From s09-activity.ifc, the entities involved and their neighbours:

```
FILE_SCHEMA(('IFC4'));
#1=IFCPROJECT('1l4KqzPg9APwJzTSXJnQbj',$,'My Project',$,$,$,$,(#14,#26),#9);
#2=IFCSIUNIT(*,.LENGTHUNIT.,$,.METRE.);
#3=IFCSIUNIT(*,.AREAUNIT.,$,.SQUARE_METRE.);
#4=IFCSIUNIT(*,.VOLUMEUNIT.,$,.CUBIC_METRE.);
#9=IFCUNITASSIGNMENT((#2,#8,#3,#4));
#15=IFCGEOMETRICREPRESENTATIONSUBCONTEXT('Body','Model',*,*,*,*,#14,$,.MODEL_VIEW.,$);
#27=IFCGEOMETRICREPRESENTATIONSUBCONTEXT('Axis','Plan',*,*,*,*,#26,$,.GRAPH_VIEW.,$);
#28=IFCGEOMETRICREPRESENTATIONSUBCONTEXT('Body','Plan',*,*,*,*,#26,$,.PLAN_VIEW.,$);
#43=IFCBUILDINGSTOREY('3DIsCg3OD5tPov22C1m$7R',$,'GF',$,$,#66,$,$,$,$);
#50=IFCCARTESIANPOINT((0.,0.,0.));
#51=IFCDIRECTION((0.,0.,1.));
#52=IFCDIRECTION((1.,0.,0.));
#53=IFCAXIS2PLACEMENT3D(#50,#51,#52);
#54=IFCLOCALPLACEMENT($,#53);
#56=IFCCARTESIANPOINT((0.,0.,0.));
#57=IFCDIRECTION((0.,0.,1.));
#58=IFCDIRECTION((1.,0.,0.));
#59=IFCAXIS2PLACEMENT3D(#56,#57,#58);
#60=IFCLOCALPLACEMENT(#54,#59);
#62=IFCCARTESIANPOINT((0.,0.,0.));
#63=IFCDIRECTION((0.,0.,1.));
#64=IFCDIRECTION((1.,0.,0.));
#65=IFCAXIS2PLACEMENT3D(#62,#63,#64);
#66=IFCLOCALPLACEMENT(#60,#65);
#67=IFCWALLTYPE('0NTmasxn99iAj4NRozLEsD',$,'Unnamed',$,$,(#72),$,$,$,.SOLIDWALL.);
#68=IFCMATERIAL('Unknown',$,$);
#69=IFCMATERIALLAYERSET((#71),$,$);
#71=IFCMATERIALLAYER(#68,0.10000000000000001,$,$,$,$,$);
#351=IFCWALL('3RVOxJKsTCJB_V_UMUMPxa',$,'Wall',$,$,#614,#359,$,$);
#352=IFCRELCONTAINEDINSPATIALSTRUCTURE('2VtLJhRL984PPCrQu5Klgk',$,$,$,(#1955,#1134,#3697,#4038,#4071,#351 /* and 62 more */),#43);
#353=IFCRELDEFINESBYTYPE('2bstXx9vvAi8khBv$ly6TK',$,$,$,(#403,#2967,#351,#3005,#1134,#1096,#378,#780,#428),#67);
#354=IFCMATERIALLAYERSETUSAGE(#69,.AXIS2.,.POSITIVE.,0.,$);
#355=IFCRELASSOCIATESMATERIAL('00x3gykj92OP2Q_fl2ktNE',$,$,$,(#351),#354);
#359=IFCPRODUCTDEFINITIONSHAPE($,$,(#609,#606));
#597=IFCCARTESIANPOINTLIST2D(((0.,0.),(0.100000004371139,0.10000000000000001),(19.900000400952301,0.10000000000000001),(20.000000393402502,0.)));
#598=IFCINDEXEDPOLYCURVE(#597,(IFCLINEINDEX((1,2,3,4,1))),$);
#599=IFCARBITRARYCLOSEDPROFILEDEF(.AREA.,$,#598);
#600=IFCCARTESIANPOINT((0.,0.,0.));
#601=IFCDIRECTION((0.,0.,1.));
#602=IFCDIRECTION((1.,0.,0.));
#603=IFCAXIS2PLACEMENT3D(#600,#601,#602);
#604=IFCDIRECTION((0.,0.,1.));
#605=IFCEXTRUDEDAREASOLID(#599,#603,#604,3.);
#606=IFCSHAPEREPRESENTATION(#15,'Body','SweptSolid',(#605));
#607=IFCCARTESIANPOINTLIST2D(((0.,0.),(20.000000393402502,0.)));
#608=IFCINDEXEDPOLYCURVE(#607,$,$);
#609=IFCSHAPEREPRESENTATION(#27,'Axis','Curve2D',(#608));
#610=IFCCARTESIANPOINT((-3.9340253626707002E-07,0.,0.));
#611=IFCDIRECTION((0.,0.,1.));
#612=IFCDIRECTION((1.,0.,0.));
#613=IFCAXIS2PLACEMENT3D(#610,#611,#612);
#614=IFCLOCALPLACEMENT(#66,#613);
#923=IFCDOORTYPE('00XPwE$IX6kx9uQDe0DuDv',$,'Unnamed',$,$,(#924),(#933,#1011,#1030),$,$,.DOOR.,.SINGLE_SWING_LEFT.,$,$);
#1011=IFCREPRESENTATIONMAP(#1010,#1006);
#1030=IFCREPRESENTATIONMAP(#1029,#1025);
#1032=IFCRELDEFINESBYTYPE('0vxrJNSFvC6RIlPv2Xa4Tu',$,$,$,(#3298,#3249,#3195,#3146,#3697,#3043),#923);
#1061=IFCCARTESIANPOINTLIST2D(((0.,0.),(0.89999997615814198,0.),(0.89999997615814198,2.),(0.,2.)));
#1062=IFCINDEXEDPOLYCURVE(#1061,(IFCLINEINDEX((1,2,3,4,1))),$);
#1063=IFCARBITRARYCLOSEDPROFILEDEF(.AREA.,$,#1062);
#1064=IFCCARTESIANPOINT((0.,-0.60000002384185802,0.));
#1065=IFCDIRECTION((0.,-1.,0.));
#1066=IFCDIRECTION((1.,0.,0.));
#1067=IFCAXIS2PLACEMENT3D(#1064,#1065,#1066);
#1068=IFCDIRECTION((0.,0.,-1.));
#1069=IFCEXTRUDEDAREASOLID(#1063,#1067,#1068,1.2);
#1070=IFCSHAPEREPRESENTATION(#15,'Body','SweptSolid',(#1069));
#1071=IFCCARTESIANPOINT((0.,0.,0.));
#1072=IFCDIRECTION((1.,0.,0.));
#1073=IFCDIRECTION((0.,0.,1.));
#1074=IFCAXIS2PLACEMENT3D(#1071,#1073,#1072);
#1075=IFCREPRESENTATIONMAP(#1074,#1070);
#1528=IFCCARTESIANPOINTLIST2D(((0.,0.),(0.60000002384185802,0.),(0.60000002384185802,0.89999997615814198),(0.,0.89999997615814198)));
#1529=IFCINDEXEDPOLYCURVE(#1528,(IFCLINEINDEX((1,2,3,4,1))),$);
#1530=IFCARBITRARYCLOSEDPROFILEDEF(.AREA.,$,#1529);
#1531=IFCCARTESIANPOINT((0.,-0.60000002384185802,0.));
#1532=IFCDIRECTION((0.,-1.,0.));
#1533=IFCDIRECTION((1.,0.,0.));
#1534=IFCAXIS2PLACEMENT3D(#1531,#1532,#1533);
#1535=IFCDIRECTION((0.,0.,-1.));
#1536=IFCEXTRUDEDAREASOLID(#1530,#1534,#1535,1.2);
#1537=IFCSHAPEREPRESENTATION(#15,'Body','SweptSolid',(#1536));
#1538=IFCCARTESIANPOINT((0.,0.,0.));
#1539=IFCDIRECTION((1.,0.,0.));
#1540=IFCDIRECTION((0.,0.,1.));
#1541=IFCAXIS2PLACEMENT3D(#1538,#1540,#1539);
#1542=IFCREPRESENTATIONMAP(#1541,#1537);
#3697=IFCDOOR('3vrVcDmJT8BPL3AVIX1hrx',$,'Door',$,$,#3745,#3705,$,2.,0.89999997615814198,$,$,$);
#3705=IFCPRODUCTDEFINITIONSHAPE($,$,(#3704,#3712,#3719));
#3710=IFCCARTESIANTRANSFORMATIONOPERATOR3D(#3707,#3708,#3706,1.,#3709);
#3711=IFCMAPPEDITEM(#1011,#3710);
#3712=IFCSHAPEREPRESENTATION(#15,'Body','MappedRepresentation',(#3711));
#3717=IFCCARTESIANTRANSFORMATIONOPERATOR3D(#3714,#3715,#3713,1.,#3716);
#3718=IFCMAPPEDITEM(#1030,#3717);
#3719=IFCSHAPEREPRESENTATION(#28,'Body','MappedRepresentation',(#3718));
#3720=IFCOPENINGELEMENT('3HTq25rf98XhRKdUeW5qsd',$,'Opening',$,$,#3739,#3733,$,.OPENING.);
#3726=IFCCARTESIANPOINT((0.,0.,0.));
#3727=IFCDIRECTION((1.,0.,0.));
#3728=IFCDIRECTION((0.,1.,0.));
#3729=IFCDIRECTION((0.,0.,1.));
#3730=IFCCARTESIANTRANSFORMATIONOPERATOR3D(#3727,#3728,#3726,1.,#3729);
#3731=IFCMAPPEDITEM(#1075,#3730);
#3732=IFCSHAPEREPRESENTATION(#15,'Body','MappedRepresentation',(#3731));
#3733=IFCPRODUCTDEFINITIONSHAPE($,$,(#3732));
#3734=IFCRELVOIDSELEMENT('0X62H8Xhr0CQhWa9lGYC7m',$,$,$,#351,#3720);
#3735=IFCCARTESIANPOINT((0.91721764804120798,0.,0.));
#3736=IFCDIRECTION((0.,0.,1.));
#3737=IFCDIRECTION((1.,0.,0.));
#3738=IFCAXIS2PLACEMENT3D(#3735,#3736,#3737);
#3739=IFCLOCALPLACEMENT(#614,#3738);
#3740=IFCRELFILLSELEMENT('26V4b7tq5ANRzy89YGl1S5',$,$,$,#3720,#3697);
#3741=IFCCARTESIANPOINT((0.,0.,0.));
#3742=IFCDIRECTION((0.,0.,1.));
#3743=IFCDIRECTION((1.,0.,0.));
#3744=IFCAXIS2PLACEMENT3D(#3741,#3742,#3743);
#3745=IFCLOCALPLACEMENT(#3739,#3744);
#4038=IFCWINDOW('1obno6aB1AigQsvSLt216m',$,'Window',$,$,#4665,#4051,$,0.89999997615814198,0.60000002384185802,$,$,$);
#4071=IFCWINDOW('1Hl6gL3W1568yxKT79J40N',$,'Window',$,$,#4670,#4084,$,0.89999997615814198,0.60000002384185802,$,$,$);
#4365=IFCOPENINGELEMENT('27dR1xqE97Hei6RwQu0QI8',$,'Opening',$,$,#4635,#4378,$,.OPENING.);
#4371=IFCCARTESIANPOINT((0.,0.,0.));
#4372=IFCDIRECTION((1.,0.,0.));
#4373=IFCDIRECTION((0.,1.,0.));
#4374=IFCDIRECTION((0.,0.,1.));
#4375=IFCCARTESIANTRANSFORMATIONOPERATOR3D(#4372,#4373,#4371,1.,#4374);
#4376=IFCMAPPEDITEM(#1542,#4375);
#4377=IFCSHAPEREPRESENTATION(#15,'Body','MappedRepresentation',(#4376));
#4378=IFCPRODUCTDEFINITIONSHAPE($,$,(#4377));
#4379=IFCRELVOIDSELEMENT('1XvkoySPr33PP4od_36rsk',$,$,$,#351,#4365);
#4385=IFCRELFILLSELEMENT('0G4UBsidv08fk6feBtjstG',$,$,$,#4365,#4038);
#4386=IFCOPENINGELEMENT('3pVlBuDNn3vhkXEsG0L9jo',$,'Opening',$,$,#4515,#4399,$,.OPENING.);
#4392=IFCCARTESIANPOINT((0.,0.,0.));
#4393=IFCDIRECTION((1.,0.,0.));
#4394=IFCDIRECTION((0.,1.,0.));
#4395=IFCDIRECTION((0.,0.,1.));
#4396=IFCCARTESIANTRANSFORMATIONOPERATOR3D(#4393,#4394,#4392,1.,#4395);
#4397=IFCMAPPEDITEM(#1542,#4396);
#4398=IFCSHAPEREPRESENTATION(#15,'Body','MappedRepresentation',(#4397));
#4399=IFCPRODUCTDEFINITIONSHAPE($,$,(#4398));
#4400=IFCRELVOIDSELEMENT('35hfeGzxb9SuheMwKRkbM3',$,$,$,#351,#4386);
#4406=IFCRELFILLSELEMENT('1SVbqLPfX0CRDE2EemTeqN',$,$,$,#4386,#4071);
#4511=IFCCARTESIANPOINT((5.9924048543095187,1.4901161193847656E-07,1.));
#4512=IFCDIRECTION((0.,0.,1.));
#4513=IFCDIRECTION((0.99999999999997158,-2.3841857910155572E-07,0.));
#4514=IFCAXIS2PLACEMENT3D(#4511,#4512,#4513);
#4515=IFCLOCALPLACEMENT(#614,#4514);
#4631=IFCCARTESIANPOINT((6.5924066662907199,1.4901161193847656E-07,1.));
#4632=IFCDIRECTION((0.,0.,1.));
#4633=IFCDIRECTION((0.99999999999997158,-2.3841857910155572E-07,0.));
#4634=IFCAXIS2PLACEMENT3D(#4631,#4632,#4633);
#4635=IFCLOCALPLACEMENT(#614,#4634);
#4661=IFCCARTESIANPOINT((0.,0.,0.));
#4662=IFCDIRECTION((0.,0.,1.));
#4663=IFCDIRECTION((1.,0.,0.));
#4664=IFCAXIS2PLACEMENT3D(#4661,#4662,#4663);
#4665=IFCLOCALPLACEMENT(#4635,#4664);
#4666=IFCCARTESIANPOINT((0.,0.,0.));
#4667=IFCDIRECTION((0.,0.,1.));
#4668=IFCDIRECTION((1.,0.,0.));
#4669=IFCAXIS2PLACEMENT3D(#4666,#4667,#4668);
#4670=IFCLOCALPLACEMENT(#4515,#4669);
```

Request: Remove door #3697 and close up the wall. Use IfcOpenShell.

```python
import ifcopenshell
import ifcopenshell.api.feature
import ifcopenshell.api.root
import ifcopenshell.geom
import ifcopenshell.util.shape

model = ifcopenshell.open("s09-activity.ifc")
settings = ifcopenshell.geom.settings()


def volume(element):
    """Net volume in cubic metres, openings subtracted."""
    shape = ifcopenshell.geom.create_shape(settings, element)
    return ifcopenshell.util.shape.get_volume(shape.geometry)


door = model.by_guid("3vrVcDmJT8BPL3AVIX1hrx")
opening = door.FillsVoids[0].RelatingOpeningElement
wall = opening.VoidsElements[0].RelatingBuildingElement
before = volume(wall)

ifcopenshell.api.root.remove_product(model, product=door)
ifcopenshell.api.feature.remove_feature(model, feature=opening)

after = volume(wall)

print(f"wall volume {before:.3f} -> {after:.3f} m3")

model.write("s09-activity-out.ifc")
```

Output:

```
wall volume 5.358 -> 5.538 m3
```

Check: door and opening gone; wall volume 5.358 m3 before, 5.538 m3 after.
